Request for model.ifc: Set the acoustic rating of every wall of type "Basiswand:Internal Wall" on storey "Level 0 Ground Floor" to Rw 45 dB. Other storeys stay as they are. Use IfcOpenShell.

First a look at what the model holds.

```python
import ifcopenshell
import ifcopenshell.util.element

model = ifcopenshell.open("model.ifc")
print(model.schema)
storey = next(s for s in model.by_type("IfcBuildingStorey") if s.Name == "Level 0 Ground Floor")
walls = [e for e in ifcopenshell.util.element.get_decomposition(storey) if e.is_a("IfcWall")]
seen = {}
for e in walls:
    element_type = ifcopenshell.util.element.get_type(e)
    key = (element_type.Name if element_type != e and element_type else None, ifcopenshell.util.element.get_pset(e, "Pset_WallCommon", "AcousticRating"))
    seen[key] = seen.get(key, 0) + 1
for (name, value), count in sorted(seen.items(), key=str):
    print(count, "x", name, "|", value)
```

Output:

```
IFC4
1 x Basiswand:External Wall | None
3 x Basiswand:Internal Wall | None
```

```python
import ifcopenshell
import ifcopenshell.api.pset
import ifcopenshell.util.element

model = ifcopenshell.open("model.ifc")

storey = next(s for s in model.by_type("IfcBuildingStorey") if s.Name == "Level 0 Ground Floor")
walls = [e for e in ifcopenshell.util.element.get_decomposition(storey) if e.is_a("IfcWall")]

count = 0
for e in walls:
    element_type = ifcopenshell.util.element.get_type(e)
    if element_type in (None, e) or element_type.Name != "Basiswand:Internal Wall":
        continue
    # add_pset returns the element's existing set when there is one.
    pset = ifcopenshell.api.pset.add_pset(model, product=e, name="Pset_WallCommon")
    ifcopenshell.api.pset.edit_pset(model, pset=pset, properties={"AcousticRating": "Rw 45 dB"})
    count += 1

print(count, "walls updated")

model.write("model_edited.ifc")
```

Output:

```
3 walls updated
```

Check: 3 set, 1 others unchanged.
